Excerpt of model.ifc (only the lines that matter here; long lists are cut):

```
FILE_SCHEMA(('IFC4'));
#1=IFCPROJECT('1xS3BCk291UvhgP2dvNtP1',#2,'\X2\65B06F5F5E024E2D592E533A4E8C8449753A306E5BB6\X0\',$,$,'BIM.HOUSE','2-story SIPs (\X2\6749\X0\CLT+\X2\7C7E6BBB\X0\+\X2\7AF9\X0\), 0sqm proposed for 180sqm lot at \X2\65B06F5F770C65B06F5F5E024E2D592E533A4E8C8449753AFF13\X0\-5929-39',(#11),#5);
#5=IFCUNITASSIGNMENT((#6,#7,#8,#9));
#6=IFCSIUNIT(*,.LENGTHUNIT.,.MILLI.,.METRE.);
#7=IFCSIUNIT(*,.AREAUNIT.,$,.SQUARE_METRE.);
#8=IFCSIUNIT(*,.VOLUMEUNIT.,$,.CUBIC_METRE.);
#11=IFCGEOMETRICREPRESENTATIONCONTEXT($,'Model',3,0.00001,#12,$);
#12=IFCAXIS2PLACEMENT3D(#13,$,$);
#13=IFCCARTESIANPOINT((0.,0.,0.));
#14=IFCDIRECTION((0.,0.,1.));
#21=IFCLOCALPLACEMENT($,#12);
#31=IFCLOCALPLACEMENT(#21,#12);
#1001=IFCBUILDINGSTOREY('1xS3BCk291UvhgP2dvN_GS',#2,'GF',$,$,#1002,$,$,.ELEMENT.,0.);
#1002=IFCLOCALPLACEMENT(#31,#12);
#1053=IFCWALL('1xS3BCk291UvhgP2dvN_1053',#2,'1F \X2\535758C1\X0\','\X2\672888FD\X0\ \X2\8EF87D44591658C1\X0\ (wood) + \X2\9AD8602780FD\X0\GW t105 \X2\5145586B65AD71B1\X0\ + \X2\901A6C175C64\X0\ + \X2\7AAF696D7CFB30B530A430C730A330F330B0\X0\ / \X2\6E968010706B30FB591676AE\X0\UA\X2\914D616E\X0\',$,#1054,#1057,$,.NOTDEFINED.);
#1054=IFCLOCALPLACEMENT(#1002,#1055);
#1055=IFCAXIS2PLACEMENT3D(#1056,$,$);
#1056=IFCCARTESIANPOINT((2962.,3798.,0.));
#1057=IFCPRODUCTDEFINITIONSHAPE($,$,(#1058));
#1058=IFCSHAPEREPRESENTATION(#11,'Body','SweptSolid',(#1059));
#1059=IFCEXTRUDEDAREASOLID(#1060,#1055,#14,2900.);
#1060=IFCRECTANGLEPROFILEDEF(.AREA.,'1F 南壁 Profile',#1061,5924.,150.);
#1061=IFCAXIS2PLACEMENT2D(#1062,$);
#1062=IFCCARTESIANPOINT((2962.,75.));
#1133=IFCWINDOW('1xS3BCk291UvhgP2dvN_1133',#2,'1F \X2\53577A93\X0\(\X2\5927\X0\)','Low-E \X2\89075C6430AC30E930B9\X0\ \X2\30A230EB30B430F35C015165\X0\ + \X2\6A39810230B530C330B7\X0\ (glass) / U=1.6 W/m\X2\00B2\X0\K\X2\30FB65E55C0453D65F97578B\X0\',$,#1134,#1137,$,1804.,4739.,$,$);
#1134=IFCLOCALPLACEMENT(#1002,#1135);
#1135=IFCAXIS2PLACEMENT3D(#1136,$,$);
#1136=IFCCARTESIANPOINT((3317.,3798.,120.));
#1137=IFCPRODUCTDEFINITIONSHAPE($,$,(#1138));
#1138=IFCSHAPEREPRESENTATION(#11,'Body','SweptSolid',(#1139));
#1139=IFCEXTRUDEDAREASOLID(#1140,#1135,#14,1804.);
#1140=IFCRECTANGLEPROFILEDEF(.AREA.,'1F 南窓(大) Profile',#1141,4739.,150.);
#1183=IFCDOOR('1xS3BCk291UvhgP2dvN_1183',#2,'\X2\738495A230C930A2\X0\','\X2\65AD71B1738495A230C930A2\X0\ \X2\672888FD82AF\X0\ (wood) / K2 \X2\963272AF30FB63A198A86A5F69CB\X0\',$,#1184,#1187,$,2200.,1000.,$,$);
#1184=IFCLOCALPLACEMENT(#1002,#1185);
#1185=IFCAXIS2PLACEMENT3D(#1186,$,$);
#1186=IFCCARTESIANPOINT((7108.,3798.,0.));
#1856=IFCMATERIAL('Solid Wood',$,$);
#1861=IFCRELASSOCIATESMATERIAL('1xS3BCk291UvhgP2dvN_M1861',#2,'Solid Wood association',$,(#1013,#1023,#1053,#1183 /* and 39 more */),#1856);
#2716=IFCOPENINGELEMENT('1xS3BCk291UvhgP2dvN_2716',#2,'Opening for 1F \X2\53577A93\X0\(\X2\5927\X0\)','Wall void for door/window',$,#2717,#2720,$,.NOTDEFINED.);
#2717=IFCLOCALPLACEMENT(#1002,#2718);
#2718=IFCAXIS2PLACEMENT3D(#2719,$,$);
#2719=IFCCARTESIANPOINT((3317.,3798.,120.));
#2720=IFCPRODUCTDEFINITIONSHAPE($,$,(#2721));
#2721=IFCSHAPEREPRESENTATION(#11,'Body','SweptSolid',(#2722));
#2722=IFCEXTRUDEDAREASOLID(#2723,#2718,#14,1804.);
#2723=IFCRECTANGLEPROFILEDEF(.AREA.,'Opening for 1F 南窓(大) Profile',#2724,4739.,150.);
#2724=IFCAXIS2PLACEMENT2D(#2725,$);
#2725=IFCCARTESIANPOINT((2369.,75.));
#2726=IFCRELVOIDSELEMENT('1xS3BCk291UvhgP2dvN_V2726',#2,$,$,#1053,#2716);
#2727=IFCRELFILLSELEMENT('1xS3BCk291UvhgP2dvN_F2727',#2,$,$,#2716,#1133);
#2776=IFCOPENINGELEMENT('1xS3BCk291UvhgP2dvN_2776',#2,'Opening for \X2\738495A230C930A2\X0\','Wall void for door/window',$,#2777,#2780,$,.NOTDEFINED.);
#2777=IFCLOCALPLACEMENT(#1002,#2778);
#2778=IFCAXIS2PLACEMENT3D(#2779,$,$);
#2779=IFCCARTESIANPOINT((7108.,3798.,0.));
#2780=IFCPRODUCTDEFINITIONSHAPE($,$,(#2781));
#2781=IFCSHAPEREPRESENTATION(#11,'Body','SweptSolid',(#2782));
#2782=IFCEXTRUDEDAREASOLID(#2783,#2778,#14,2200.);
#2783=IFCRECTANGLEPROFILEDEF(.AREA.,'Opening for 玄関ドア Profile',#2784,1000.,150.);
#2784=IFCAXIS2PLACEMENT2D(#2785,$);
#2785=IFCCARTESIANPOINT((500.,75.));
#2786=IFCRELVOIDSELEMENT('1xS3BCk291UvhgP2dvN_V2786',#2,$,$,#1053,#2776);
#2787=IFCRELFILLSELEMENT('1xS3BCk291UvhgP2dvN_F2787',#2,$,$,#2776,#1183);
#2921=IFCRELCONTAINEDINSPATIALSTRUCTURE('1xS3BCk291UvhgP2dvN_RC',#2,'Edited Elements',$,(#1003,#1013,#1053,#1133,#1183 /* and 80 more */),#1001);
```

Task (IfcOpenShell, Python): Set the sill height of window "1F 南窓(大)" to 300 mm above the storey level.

```python
import numpy as np
import ifcopenshell
import ifcopenshell.api.geometry
import ifcopenshell.geom
import ifcopenshell.util.element
import ifcopenshell.util.placement
import ifcopenshell.util.shape
import ifcopenshell.util.unit

model = ifcopenshell.open("model.ifc")
unit_scale = ifcopenshell.util.unit.calculate_unit_scale(model)

window = model.by_id(1133)
opening = window.FillsVoids[0].RelatingOpeningElement
storey = ifcopenshell.util.element.get_container(window, ifc_class="IfcBuildingStorey")
level = ifcopenshell.util.placement.get_local_placement(storey.ObjectPlacement)[2, 3]

# The opening's origin need not be at the sill, so measure its lowest point.
shape = ifcopenshell.geom.create_shape(ifcopenshell.geom.settings(), opening)
bottom = ifcopenshell.util.shape.get_shape_bottom_elevation(shape, shape.geometry) / unit_scale
dz = level + 0.3 / unit_scale - bottom

shift = np.array([0.0, 0.0, dz])
# The window is not placed relative to its opening, so move both.
for product in (opening, window):
    matrix = ifcopenshell.util.placement.get_local_placement(product.ObjectPlacement)
    matrix[:3, 3] += shift
    ifcopenshell.api.geometry.edit_object_placement(model, product=product, matrix=matrix, is_si=False)

print(f"moved by {dz * unit_scale:+.3f} m")

model.write("model_updated.ifc")
```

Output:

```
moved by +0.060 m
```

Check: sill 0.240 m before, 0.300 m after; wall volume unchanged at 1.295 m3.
